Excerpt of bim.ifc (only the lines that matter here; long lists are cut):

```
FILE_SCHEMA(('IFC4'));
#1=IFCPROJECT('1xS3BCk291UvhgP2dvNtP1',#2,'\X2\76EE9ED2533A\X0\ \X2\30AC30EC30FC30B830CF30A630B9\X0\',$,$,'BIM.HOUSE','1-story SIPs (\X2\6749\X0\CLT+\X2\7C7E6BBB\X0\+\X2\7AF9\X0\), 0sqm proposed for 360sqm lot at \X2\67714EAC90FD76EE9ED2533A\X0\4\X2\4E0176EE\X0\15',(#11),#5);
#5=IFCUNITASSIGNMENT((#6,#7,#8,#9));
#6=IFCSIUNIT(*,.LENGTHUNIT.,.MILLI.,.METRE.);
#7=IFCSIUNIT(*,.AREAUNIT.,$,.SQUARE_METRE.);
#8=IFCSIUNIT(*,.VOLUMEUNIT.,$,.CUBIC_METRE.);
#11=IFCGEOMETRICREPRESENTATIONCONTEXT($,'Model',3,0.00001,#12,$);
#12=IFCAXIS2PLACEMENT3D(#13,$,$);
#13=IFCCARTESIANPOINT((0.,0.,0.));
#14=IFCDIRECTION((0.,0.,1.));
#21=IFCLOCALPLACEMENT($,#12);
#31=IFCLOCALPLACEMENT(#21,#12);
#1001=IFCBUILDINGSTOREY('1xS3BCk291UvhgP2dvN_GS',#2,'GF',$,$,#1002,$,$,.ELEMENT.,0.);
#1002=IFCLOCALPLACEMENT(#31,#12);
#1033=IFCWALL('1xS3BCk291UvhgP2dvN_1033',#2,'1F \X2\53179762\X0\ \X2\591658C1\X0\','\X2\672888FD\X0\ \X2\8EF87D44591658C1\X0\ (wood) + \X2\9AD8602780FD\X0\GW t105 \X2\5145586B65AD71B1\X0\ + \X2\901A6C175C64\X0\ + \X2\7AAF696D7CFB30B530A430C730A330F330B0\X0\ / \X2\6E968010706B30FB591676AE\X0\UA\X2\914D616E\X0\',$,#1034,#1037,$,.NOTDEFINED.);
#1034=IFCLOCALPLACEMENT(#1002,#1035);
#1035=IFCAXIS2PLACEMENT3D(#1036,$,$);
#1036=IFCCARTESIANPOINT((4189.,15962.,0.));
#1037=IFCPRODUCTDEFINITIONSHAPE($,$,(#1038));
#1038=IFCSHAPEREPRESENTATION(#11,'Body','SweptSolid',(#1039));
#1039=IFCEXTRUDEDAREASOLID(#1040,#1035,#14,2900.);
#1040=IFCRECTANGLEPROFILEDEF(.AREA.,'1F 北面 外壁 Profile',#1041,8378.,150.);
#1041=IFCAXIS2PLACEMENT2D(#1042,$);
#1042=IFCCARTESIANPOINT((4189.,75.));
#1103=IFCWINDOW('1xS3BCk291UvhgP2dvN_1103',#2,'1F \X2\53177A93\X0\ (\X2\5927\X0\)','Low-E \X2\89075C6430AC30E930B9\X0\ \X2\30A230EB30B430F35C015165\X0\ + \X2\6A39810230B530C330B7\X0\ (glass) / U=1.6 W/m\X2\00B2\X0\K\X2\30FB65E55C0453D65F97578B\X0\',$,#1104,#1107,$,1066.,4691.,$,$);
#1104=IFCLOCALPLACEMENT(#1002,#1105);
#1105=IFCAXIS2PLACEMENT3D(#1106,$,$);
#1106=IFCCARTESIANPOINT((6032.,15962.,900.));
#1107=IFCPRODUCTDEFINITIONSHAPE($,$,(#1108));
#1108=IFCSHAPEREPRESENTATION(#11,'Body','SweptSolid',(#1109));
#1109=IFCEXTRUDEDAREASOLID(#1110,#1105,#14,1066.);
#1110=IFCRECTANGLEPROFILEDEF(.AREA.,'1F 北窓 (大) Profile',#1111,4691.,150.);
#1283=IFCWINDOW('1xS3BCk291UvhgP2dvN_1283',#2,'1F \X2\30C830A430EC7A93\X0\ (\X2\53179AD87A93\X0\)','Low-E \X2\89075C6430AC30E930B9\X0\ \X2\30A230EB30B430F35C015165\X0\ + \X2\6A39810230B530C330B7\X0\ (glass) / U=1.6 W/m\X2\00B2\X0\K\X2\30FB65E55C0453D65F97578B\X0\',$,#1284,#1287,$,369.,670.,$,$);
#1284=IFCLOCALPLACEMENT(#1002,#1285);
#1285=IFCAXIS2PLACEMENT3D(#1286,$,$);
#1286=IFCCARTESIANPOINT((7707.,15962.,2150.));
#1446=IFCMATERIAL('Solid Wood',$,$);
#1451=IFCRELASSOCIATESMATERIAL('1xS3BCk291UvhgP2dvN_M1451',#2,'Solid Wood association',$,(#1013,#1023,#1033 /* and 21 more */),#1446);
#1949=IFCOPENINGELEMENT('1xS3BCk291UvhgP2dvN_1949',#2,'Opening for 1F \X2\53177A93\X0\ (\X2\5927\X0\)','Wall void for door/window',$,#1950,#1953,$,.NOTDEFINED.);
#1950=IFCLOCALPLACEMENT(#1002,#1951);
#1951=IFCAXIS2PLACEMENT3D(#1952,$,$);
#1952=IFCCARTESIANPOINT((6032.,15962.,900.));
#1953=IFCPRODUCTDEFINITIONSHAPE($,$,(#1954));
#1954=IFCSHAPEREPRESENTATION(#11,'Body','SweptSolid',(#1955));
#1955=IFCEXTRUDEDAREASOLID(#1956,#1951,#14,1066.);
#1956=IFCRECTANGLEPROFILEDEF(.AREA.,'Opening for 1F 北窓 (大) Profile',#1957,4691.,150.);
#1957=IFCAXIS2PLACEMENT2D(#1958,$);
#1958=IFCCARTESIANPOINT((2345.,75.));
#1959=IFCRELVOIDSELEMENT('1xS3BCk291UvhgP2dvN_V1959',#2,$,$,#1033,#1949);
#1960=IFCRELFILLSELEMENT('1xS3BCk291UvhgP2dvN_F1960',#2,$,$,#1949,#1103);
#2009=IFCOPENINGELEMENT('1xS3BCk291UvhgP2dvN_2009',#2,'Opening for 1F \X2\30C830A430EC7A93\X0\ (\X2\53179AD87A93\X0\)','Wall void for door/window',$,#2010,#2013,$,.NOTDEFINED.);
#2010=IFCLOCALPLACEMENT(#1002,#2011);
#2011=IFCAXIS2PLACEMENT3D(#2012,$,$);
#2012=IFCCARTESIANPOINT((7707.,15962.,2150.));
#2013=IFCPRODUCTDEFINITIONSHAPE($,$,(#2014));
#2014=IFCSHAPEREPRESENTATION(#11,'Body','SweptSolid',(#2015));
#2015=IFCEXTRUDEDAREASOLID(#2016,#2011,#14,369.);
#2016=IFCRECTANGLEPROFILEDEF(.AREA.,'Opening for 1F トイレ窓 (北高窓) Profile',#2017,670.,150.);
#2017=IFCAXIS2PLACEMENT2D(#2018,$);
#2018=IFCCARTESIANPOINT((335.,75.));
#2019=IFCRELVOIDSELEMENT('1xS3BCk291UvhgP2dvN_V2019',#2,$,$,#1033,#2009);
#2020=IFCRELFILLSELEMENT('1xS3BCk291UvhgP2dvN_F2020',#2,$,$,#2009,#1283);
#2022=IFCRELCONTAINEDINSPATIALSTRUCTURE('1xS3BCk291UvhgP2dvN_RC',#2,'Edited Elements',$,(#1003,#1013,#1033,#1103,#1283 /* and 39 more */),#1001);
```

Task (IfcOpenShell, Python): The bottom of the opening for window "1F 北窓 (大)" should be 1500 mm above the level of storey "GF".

```python
import numpy as np
import ifcopenshell
import ifcopenshell.api.geometry
import ifcopenshell.geom
import ifcopenshell.util.element
import ifcopenshell.util.placement
import ifcopenshell.util.shape
import ifcopenshell.util.unit

model = ifcopenshell.open("bim.ifc")
unit_scale = ifcopenshell.util.unit.calculate_unit_scale(model)

window = model.by_id(1103)
opening = window.FillsVoids[0].RelatingOpeningElement
storey = ifcopenshell.util.element.get_container(window, ifc_class="IfcBuildingStorey")
level = ifcopenshell.util.placement.get_local_placement(storey.ObjectPlacement)[2, 3]

# The opening's origin need not be at the sill, so measure its lowest point.
shape = ifcopenshell.geom.create_shape(ifcopenshell.geom.settings(), opening)
bottom = ifcopenshell.util.shape.get_shape_bottom_elevation(shape, shape.geometry) / unit_scale
dz = level + 1500.0 - bottom

shift = np.array([0.0, 0.0, dz])
# The window is not placed relative to its opening, so move both.
for product in (opening, window):
    matrix = ifcopenshell.util.placement.get_local_placement(product.ObjectPlacement)
    matrix[:3, 3] += shift
    ifcopenshell.api.geometry.edit_object_placement(model, product=product, matrix=matrix, is_si=False)

print(f"moved by {dz * unit_scale:+.3f} m")

model.write("bim_rev.ifc")
```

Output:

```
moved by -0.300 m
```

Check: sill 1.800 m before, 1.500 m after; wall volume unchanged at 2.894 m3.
